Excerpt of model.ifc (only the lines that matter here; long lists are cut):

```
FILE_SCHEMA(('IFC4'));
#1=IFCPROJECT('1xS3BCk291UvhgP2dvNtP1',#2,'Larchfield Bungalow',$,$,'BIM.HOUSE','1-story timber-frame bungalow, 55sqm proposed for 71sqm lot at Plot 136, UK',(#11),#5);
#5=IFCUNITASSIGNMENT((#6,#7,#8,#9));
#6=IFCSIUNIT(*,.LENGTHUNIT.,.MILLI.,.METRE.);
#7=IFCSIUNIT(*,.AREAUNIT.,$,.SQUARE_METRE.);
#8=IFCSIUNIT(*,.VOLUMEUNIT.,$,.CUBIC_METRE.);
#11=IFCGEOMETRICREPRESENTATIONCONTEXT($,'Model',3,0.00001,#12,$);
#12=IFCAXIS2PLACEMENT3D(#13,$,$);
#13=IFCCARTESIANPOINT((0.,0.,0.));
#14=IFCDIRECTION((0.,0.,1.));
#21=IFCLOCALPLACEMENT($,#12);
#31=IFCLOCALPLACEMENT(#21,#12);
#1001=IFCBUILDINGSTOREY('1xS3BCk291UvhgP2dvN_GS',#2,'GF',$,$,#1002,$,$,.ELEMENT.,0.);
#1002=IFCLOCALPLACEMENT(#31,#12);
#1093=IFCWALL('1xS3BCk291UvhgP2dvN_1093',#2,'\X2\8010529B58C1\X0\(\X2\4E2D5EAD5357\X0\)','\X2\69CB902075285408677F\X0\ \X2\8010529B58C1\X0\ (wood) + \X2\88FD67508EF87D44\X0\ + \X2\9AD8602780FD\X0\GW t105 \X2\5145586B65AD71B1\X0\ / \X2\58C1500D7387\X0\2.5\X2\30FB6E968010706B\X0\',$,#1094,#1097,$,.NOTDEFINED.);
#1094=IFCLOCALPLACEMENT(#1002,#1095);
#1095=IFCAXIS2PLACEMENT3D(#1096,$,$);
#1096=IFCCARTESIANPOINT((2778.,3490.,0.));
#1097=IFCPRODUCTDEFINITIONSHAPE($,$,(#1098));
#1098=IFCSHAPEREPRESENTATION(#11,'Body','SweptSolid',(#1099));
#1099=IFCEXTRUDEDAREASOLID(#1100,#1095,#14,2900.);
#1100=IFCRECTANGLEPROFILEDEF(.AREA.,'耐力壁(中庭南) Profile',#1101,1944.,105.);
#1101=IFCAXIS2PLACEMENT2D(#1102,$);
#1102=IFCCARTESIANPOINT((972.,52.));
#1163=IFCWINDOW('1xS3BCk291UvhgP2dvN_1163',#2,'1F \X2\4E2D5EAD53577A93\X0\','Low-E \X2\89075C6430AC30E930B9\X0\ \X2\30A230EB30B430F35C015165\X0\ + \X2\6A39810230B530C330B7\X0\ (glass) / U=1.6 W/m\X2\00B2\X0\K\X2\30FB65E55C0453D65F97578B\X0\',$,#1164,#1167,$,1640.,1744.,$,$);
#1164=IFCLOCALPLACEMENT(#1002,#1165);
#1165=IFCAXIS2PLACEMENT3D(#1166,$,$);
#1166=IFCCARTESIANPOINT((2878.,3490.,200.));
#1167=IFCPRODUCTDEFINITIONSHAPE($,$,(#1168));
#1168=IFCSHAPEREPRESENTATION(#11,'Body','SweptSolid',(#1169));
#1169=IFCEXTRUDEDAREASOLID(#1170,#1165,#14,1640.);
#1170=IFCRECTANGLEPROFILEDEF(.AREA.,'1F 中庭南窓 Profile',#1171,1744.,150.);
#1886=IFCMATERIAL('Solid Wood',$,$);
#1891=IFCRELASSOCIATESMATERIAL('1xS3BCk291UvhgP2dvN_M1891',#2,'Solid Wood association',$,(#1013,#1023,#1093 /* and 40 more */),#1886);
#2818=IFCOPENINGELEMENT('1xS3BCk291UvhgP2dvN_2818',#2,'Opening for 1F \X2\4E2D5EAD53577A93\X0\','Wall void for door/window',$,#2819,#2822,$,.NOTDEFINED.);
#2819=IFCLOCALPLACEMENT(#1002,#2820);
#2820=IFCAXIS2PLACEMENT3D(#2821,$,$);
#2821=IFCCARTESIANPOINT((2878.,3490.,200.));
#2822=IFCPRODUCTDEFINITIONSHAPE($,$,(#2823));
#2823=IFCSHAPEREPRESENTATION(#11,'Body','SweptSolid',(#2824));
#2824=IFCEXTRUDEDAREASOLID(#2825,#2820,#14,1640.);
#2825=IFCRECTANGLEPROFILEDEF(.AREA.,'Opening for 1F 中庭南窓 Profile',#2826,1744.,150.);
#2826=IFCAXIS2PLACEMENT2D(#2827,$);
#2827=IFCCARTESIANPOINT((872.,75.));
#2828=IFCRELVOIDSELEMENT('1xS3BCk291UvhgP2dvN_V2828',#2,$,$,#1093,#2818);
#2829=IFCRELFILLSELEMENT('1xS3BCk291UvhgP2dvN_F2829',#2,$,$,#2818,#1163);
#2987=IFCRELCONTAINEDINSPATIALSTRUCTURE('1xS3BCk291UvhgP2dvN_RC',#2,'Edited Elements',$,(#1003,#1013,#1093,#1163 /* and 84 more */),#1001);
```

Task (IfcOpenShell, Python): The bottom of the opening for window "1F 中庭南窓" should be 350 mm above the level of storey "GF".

```python
import numpy as np
import ifcopenshell
import ifcopenshell.api.geometry
import ifcopenshell.geom
import ifcopenshell.util.element
import ifcopenshell.util.placement
import ifcopenshell.util.shape
import ifcopenshell.util.unit

model = ifcopenshell.open("model.ifc")
unit_scale = ifcopenshell.util.unit.calculate_unit_scale(model)

window = model.by_guid("1xS3BCk291UvhgP2dvN_1163")
opening = window.FillsVoids[0].RelatingOpeningElement
storey = ifcopenshell.util.element.get_container(window, ifc_class="IfcBuildingStorey")
level = ifcopenshell.util.placement.get_local_placement(storey.ObjectPlacement)[2, 3]

# The opening's origin need not be at the sill, so measure its lowest point.
shape = ifcopenshell.geom.create_shape(ifcopenshell.geom.settings(), opening)
bottom = ifcopenshell.util.shape.get_shape_bottom_elevation(shape, shape.geometry) / unit_scale
dz = level + 350.0 - bottom

shift = np.array([0.0, 0.0, dz])
# The window is not placed relative to its opening, so move both.
for product in (opening, window):
    matrix = ifcopenshell.util.placement.get_local_placement(product.ObjectPlacement)
    matrix[:3, 3] += shift
    ifcopenshell.api.geometry.edit_object_placement(model, product=product, matrix=matrix, is_si=False)

print(f"moved by {dz * unit_scale:+.3f} m")

model.write("model-out.ifc")
```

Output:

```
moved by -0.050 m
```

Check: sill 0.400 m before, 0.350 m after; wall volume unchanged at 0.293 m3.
